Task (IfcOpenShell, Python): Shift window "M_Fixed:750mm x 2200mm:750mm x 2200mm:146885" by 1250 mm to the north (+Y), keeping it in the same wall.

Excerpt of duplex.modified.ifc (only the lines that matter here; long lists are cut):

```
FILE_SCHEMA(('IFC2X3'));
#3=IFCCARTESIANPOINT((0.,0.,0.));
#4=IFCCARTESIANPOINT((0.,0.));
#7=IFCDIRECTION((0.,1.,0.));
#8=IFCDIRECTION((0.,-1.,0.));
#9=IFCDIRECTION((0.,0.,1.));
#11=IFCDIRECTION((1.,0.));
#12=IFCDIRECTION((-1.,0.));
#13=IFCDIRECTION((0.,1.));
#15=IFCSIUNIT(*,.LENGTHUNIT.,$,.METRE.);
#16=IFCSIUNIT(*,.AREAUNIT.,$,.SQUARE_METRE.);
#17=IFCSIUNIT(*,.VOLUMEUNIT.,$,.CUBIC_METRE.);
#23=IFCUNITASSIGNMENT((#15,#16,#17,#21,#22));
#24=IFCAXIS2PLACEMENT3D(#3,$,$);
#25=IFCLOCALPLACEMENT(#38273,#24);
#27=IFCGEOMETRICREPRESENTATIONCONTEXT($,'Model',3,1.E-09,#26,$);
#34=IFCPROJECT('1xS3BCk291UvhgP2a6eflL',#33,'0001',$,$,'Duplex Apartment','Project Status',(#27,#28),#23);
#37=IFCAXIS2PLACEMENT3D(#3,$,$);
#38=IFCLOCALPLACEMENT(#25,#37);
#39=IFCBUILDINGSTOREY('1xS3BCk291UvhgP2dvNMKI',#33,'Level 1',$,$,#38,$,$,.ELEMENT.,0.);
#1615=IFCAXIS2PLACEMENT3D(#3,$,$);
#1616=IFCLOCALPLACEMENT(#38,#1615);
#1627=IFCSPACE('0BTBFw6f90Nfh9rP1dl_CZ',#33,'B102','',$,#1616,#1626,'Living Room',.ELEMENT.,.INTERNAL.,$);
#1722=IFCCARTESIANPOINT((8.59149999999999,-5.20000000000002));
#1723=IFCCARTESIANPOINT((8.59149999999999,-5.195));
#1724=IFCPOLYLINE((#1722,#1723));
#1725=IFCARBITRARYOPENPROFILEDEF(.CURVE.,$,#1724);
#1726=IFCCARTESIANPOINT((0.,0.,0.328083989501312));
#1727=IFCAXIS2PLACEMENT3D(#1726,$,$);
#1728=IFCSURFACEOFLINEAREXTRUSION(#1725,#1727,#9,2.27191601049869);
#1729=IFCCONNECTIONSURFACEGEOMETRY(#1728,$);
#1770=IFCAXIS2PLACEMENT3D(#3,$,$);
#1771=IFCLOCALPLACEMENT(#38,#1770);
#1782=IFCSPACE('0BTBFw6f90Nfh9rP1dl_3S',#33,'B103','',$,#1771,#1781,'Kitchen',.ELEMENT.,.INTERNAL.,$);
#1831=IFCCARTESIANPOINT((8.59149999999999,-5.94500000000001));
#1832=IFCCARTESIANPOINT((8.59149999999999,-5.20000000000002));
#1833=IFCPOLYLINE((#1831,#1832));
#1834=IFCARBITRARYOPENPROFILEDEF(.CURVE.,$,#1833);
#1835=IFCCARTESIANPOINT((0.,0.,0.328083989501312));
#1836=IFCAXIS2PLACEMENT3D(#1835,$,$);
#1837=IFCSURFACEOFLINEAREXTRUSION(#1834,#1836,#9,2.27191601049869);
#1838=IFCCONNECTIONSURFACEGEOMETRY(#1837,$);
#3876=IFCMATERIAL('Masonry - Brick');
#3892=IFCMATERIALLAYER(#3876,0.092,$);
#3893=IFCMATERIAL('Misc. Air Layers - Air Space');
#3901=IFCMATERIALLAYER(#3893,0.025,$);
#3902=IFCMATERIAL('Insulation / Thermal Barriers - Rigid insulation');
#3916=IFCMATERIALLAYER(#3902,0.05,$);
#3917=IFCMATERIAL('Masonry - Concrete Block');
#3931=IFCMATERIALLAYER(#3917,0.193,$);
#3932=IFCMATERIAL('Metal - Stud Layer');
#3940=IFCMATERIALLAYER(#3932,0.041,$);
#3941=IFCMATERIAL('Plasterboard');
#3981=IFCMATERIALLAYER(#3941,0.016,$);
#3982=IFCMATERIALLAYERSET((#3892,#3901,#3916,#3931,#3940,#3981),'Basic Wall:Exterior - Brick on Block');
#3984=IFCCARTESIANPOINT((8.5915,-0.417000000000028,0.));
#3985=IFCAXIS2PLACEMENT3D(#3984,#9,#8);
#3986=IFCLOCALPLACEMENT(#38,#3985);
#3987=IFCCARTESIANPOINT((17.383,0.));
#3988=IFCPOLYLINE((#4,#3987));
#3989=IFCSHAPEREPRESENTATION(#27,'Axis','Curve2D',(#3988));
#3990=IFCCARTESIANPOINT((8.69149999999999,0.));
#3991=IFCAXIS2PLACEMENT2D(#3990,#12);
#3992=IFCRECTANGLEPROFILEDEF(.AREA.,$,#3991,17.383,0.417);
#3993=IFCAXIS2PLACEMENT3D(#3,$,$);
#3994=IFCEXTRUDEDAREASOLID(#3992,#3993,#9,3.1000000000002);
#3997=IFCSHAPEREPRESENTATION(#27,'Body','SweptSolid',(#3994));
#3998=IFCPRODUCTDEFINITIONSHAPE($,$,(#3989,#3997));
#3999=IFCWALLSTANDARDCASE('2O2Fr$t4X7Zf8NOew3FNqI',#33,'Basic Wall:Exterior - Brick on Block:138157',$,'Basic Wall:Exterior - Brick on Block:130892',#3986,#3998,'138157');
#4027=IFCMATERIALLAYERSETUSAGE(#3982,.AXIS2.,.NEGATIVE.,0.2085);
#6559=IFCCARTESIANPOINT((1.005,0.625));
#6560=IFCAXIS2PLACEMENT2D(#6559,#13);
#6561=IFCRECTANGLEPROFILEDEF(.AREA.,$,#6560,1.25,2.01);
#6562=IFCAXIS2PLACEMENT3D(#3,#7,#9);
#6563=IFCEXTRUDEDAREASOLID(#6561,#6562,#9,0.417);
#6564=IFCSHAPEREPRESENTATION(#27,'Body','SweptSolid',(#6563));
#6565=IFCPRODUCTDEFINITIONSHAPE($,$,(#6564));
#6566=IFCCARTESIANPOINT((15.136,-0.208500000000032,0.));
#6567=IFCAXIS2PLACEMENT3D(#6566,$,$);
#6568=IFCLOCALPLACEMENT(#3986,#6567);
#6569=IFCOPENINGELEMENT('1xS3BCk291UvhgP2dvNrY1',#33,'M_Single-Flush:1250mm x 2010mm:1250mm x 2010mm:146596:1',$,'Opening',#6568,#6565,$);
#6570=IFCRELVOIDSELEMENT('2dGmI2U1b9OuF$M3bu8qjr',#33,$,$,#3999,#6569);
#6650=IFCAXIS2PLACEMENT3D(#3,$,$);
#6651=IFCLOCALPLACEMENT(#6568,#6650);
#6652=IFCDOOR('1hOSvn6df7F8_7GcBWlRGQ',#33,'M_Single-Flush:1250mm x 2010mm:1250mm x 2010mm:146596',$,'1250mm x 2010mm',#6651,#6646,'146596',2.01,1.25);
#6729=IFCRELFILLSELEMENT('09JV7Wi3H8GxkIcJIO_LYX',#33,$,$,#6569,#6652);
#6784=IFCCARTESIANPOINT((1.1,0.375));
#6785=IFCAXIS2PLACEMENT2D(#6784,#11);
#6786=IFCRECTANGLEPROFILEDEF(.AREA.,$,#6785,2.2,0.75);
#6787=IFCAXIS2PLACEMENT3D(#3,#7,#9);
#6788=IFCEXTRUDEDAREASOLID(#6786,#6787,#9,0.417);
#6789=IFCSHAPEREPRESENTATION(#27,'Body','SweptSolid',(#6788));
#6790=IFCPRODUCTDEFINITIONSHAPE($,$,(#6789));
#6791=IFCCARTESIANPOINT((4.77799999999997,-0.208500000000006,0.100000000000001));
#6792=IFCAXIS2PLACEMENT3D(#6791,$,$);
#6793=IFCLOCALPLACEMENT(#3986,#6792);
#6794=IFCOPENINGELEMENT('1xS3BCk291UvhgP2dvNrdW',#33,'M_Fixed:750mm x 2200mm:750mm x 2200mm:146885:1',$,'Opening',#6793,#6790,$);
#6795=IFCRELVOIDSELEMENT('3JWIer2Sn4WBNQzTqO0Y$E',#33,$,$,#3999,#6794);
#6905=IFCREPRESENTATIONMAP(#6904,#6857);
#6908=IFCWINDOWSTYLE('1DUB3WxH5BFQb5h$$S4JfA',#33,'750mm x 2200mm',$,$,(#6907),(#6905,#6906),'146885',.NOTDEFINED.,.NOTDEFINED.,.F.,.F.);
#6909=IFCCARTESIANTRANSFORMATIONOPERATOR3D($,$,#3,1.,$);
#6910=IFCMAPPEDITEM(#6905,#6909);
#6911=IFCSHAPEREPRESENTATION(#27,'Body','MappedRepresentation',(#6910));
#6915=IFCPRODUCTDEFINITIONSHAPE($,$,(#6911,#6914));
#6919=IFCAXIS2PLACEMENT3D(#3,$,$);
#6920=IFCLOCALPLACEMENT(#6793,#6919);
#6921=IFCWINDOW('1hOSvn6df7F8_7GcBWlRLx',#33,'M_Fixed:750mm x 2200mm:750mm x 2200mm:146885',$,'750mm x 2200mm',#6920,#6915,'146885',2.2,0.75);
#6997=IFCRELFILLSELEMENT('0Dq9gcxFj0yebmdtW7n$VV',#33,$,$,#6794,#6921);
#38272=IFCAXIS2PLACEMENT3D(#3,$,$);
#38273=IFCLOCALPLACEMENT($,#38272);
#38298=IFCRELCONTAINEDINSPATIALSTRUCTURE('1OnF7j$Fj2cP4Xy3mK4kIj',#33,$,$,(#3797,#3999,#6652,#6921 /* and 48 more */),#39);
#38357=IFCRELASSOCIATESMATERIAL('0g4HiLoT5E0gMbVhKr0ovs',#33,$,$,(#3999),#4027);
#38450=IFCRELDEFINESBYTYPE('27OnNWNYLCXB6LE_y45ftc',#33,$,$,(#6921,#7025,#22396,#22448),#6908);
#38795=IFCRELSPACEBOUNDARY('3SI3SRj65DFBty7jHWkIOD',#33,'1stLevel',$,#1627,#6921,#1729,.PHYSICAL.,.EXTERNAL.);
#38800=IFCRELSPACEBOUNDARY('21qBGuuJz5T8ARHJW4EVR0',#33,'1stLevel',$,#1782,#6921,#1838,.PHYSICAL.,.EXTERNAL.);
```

```python
import numpy as np
import ifcopenshell
import ifcopenshell.api.geometry
import ifcopenshell.util.placement
import ifcopenshell.util.unit

model = ifcopenshell.open("duplex.modified.ifc")
unit_scale = ifcopenshell.util.unit.calculate_unit_scale(model)

window = model.by_guid("1hOSvn6df7F8_7GcBWlRLx")
opening = window.FillsVoids[0].RelatingOpeningElement
wall = opening.VoidsElements[0].RelatingBuildingElement

wall_matrix = ifcopenshell.util.placement.get_local_placement(wall.ObjectPlacement)
shift = wall_matrix[:3, 0] * -1.25 / unit_scale
before = ifcopenshell.util.placement.get_local_placement(window.ObjectPlacement)[:3, 3].copy()

# The window is placed relative to its opening, so it follows when the opening moves.
matrix = ifcopenshell.util.placement.get_local_placement(opening.ObjectPlacement)
matrix[:3, 3] += shift
ifcopenshell.api.geometry.edit_object_placement(
    model, product=opening, matrix=matrix, is_si=False, should_transform_children=True
)

# Space boundary surfaces are stored in each space's coordinates; move them too.
for rel in window.ProvidesBoundaries:
    if not rel.ConnectionGeometry:
        continue
    surface = rel.ConnectionGeometry.SurfaceOnRelatingElement
    space_matrix = ifcopenshell.util.placement.get_local_placement(rel.RelatingSpace.ObjectPlacement)
    point = np.array(surface.Position.Location.Coordinates) + space_matrix[:3, :3].T @ shift
    surface.Position = model.createIfcAxis2Placement3D(
        model.createIfcCartesianPoint(point.tolist()), surface.Position.Axis, surface.Position.RefDirection
    )

after = ifcopenshell.util.placement.get_local_placement(window.ObjectPlacement)[:3, 3]
print("window moved by", (after - before).round(3) + 0.0)

model.write("duplex.modified-out.ifc")
```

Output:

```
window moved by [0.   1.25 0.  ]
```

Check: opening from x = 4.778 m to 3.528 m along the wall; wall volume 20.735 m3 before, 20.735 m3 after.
